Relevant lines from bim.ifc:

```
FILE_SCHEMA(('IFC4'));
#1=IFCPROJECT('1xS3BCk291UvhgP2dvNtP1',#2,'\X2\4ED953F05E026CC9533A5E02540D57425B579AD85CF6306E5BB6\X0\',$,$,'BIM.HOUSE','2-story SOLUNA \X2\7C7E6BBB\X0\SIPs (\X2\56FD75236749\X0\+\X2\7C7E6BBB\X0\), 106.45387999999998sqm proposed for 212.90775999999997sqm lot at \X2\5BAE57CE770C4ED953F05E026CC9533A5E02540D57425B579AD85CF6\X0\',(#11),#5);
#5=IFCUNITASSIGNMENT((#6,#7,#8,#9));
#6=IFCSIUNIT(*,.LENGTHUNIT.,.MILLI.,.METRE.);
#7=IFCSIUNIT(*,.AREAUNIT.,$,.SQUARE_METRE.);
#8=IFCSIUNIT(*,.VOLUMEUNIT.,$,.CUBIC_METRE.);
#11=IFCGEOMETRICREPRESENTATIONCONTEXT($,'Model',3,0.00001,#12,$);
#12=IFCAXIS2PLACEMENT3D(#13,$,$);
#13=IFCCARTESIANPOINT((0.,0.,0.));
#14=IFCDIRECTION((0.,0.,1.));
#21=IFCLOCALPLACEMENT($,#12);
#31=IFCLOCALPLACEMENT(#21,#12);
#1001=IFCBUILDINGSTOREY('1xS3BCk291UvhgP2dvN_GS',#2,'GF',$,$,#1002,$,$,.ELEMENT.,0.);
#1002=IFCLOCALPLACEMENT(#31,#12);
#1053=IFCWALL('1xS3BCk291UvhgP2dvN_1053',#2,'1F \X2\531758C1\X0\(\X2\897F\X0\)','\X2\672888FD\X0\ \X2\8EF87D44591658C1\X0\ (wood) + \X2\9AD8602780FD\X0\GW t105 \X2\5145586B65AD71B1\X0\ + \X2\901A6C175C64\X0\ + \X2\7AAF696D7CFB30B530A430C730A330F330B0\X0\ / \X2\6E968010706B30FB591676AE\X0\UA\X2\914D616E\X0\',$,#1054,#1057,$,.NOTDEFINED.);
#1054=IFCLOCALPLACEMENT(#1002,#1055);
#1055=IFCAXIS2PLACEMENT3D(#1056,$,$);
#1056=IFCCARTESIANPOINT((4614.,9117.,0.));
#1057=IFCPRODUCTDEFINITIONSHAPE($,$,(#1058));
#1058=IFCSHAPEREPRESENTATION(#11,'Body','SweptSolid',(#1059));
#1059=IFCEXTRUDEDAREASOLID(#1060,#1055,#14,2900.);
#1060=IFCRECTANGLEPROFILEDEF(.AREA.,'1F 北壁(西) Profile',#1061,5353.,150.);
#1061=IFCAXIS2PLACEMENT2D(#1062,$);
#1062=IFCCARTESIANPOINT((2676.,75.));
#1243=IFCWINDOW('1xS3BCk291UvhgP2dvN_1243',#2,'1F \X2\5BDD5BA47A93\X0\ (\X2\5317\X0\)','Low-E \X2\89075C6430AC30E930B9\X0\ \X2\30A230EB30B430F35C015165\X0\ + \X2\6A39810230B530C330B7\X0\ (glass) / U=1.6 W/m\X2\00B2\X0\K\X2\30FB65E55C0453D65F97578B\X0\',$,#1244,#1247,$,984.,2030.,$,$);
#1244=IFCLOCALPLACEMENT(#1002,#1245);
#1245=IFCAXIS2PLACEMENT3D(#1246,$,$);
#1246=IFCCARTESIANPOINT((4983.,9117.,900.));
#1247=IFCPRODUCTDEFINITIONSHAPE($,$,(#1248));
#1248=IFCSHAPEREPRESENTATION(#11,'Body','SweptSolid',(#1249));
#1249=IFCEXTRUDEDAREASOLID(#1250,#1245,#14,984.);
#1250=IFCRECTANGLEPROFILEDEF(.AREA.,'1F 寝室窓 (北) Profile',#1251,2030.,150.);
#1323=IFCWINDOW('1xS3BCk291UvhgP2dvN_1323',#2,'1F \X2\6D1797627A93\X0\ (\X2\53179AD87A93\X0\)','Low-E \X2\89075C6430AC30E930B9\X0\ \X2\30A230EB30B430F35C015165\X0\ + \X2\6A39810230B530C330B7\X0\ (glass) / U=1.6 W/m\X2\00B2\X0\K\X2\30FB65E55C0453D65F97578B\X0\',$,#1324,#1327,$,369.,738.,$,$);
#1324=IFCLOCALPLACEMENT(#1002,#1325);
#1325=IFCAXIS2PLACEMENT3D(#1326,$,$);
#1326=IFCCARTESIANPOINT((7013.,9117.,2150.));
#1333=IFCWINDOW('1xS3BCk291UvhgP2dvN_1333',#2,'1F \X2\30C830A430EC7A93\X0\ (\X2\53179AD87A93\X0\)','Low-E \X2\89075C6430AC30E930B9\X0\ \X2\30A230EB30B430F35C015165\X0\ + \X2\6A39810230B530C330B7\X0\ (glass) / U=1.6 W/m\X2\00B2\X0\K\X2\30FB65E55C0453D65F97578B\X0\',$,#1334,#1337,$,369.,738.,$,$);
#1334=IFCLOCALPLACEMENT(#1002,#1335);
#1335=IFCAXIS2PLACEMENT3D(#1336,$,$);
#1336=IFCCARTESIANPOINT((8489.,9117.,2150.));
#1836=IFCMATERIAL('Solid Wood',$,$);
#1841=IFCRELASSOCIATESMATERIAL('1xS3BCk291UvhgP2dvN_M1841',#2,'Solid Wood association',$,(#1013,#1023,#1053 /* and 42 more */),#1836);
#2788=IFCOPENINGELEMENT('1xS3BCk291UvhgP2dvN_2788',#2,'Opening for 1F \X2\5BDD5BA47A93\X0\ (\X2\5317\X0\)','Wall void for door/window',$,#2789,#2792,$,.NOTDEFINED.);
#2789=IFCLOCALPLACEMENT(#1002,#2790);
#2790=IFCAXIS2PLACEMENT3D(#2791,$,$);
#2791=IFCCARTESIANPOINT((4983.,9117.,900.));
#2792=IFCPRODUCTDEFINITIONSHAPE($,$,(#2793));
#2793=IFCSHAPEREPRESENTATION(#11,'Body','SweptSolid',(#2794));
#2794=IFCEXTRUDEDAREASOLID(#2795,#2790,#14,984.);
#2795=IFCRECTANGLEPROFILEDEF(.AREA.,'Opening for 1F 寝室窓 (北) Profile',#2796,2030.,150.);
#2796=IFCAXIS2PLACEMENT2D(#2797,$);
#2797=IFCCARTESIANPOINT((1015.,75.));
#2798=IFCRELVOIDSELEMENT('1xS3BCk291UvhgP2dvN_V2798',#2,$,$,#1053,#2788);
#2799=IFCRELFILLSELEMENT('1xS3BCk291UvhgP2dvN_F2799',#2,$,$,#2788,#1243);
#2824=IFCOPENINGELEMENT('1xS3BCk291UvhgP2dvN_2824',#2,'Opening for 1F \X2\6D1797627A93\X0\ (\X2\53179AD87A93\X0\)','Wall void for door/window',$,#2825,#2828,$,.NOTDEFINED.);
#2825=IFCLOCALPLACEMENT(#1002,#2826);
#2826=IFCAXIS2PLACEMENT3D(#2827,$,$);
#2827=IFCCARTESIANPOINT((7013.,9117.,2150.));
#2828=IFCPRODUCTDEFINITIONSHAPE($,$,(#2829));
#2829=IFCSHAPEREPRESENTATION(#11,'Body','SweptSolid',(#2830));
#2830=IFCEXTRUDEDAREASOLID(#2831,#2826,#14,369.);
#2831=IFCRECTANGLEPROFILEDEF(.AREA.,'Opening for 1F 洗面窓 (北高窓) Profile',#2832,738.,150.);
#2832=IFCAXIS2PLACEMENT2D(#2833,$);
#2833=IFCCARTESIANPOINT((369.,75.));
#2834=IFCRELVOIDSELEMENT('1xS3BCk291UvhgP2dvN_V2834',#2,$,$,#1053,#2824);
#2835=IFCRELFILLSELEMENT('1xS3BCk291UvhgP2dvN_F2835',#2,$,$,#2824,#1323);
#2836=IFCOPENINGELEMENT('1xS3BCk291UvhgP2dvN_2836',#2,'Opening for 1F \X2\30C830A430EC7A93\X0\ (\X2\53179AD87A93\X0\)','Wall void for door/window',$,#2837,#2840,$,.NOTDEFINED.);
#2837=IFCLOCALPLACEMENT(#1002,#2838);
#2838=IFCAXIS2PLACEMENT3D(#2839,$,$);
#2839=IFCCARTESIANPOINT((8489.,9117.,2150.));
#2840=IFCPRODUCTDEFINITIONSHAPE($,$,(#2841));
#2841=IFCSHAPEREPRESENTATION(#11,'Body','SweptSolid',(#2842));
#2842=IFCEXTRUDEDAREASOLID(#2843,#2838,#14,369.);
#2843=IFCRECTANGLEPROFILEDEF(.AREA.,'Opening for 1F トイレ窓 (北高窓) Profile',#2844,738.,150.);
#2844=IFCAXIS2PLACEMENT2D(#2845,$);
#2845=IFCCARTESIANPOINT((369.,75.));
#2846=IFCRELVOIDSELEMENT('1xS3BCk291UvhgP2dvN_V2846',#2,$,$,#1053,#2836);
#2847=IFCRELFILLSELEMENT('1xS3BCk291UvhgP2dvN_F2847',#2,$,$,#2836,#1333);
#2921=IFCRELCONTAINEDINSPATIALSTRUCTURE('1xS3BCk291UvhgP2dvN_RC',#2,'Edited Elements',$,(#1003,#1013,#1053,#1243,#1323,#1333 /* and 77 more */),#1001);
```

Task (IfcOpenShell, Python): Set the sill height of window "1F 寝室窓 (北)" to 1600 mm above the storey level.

```python
import numpy as np
import ifcopenshell
import ifcopenshell.api.geometry
import ifcopenshell.geom
import ifcopenshell.util.element
import ifcopenshell.util.placement
import ifcopenshell.util.shape
import ifcopenshell.util.unit

model = ifcopenshell.open("bim.ifc")
unit_scale = ifcopenshell.util.unit.calculate_unit_scale(model)

window = model.by_guid("1xS3BCk291UvhgP2dvN_1243")
opening = window.FillsVoids[0].RelatingOpeningElement
storey = ifcopenshell.util.element.get_container(window, ifc_class="IfcBuildingStorey")
level = ifcopenshell.util.placement.get_local_placement(storey.ObjectPlacement)[2, 3]

# The opening's origin need not be at the sill, so measure its lowest point.
shape = ifcopenshell.geom.create_shape(ifcopenshell.geom.settings(), opening)
bottom = ifcopenshell.util.shape.get_shape_bottom_elevation(shape, shape.geometry) / unit_scale
dz = level + 1.6 / unit_scale - bottom

shift = np.array([0.0, 0.0, dz])
# The window is not placed relative to its opening, so move both.
for product in (opening, window):
    matrix = ifcopenshell.util.placement.get_local_placement(product.ObjectPlacement)
    matrix[:3, 3] += shift
    ifcopenshell.api.geometry.edit_object_placement(model, product=product, matrix=matrix, is_si=False)

print(f"moved by {dz * unit_scale:+.3f} m")

model.write("bim_edited.ifc")
```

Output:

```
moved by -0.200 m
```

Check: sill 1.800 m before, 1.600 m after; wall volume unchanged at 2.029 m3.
